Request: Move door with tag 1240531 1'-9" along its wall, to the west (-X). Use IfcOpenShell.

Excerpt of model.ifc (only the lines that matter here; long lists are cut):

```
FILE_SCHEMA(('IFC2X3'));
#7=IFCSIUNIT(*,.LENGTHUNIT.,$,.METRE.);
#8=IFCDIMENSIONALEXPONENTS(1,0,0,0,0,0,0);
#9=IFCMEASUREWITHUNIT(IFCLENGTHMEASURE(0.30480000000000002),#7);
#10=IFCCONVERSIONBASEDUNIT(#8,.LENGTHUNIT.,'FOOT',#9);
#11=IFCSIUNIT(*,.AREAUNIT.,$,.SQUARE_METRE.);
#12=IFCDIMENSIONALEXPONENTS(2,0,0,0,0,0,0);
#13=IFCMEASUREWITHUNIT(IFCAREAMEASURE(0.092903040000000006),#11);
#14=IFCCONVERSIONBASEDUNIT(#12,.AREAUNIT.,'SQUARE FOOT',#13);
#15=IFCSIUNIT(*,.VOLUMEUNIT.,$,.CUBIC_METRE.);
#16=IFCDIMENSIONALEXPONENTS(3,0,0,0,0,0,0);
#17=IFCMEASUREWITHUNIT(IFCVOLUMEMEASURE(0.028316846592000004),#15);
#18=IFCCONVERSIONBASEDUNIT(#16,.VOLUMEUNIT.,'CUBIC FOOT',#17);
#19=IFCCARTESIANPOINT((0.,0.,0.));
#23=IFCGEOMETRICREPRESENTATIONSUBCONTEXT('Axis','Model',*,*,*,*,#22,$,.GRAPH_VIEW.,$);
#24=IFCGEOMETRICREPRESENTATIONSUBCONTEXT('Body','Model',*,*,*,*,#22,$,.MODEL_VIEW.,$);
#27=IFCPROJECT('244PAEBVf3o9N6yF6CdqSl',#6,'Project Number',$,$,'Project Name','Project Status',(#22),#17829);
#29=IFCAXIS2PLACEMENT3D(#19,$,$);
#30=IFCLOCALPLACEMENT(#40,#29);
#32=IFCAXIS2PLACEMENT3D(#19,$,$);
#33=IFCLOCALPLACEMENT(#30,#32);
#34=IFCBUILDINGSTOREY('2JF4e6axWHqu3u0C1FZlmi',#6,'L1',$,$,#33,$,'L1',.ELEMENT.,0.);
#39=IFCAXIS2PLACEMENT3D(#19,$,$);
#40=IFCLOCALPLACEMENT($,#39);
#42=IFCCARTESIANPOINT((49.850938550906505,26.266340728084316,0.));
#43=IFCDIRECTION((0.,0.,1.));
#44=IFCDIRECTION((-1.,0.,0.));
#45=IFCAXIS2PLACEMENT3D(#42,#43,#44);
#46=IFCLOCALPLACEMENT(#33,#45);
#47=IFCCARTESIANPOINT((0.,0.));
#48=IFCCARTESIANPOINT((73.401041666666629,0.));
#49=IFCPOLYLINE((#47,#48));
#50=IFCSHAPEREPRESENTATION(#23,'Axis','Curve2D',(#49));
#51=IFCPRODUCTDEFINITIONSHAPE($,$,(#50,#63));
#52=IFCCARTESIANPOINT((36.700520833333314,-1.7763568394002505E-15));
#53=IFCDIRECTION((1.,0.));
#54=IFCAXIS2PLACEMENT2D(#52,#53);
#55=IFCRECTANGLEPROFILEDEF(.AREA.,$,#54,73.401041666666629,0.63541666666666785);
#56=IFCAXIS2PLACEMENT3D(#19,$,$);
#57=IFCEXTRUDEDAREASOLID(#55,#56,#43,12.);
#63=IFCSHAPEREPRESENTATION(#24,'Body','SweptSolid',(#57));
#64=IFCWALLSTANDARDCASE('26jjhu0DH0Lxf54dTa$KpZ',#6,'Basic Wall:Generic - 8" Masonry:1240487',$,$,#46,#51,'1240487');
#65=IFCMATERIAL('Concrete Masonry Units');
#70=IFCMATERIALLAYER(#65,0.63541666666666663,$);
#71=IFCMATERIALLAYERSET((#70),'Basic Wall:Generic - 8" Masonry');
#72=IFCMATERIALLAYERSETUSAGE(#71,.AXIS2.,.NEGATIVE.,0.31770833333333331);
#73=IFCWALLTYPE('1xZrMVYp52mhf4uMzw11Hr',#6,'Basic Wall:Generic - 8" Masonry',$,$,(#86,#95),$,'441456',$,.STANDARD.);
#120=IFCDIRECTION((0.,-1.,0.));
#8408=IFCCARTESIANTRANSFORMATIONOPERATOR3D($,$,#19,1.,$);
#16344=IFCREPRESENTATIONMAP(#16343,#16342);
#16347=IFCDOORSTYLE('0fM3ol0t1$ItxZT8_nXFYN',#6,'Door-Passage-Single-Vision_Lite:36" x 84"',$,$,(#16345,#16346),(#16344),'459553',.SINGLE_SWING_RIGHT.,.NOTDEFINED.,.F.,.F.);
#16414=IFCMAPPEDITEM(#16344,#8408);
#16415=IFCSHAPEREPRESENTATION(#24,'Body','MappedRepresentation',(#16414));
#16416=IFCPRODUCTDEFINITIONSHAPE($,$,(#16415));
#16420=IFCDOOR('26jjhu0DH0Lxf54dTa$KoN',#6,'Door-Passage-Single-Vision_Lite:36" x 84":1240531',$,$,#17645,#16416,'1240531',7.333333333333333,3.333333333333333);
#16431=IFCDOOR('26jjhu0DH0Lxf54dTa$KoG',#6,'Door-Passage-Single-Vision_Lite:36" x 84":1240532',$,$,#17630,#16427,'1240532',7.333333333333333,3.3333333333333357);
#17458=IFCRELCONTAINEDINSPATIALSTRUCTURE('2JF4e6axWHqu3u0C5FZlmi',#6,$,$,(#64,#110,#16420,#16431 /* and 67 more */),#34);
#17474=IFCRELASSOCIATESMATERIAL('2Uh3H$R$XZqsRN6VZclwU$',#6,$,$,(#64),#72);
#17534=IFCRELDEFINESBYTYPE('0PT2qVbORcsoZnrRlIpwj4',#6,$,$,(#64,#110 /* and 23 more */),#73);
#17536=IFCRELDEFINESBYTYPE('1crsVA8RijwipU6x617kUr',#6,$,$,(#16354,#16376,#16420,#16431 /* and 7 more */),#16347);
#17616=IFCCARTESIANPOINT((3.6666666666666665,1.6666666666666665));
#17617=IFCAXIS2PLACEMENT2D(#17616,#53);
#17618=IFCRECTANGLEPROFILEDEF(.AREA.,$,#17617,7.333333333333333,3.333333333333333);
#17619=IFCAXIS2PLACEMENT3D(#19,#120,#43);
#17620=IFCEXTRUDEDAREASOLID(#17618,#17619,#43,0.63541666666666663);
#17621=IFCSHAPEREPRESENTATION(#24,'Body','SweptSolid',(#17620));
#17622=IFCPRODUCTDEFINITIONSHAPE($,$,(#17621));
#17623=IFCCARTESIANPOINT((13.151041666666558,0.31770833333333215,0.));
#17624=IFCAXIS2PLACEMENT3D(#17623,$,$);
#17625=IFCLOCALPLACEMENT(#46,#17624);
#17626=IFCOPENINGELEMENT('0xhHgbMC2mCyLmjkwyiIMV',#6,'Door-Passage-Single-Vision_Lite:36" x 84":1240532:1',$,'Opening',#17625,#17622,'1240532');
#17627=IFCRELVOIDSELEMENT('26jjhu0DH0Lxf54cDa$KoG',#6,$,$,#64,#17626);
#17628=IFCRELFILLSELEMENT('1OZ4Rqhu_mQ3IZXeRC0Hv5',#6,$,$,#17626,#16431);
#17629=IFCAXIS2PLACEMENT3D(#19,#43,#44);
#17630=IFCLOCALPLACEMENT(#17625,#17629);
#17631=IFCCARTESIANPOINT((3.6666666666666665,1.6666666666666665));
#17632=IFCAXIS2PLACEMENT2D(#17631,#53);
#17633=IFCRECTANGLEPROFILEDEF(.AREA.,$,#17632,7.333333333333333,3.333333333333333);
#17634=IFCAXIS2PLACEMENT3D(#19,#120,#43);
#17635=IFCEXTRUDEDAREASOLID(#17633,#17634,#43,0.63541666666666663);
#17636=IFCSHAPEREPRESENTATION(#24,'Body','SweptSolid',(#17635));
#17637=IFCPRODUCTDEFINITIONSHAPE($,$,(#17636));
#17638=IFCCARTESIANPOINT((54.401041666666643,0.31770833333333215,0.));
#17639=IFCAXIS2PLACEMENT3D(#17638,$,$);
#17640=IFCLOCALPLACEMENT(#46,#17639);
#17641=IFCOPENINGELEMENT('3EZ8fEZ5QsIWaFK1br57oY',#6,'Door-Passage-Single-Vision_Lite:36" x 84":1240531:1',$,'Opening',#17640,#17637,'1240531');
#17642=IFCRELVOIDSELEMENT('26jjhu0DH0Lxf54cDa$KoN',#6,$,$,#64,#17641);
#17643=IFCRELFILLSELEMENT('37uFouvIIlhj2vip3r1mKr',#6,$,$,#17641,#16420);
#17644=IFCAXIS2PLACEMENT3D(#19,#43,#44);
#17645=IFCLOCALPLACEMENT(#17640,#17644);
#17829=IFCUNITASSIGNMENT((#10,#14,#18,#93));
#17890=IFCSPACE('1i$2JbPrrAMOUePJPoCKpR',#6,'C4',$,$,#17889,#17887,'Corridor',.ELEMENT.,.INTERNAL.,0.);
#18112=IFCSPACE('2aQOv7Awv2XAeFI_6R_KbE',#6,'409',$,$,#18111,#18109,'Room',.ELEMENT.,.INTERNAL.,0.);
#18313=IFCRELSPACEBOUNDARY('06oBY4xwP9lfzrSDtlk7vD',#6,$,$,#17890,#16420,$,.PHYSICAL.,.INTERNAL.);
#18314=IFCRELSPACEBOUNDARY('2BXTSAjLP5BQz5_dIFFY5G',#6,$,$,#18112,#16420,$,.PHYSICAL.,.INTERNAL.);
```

```python
import ifcopenshell
import ifcopenshell.api.geometry
import ifcopenshell.util.placement
import ifcopenshell.util.unit

model = ifcopenshell.open("model.ifc")
unit_scale = ifcopenshell.util.unit.calculate_unit_scale(model)

door = model.by_guid("26jjhu0DH0Lxf54dTa$KoN")
opening = door.FillsVoids[0].RelatingOpeningElement
wall = opening.VoidsElements[0].RelatingBuildingElement

wall_matrix = ifcopenshell.util.placement.get_local_placement(wall.ObjectPlacement)
shift = wall_matrix[:3, 0] * 21 * 0.0254 / unit_scale
before = ifcopenshell.util.placement.get_local_placement(door.ObjectPlacement)[:3, 3].copy()

# The door is placed relative to its opening, so it follows when the opening moves.
matrix = ifcopenshell.util.placement.get_local_placement(opening.ObjectPlacement)
matrix[:3, 3] += shift
ifcopenshell.api.geometry.edit_object_placement(
    model, product=opening, matrix=matrix, is_si=False, should_transform_children=True
)

after = ifcopenshell.util.placement.get_local_placement(door.ObjectPlacement)[:3, 3]
print("door moved by", (after - before).round(3) + 0.0)

model.write("model_rev.ifc")
```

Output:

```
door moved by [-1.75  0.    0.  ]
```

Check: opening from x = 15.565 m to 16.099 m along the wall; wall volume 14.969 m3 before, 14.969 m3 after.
